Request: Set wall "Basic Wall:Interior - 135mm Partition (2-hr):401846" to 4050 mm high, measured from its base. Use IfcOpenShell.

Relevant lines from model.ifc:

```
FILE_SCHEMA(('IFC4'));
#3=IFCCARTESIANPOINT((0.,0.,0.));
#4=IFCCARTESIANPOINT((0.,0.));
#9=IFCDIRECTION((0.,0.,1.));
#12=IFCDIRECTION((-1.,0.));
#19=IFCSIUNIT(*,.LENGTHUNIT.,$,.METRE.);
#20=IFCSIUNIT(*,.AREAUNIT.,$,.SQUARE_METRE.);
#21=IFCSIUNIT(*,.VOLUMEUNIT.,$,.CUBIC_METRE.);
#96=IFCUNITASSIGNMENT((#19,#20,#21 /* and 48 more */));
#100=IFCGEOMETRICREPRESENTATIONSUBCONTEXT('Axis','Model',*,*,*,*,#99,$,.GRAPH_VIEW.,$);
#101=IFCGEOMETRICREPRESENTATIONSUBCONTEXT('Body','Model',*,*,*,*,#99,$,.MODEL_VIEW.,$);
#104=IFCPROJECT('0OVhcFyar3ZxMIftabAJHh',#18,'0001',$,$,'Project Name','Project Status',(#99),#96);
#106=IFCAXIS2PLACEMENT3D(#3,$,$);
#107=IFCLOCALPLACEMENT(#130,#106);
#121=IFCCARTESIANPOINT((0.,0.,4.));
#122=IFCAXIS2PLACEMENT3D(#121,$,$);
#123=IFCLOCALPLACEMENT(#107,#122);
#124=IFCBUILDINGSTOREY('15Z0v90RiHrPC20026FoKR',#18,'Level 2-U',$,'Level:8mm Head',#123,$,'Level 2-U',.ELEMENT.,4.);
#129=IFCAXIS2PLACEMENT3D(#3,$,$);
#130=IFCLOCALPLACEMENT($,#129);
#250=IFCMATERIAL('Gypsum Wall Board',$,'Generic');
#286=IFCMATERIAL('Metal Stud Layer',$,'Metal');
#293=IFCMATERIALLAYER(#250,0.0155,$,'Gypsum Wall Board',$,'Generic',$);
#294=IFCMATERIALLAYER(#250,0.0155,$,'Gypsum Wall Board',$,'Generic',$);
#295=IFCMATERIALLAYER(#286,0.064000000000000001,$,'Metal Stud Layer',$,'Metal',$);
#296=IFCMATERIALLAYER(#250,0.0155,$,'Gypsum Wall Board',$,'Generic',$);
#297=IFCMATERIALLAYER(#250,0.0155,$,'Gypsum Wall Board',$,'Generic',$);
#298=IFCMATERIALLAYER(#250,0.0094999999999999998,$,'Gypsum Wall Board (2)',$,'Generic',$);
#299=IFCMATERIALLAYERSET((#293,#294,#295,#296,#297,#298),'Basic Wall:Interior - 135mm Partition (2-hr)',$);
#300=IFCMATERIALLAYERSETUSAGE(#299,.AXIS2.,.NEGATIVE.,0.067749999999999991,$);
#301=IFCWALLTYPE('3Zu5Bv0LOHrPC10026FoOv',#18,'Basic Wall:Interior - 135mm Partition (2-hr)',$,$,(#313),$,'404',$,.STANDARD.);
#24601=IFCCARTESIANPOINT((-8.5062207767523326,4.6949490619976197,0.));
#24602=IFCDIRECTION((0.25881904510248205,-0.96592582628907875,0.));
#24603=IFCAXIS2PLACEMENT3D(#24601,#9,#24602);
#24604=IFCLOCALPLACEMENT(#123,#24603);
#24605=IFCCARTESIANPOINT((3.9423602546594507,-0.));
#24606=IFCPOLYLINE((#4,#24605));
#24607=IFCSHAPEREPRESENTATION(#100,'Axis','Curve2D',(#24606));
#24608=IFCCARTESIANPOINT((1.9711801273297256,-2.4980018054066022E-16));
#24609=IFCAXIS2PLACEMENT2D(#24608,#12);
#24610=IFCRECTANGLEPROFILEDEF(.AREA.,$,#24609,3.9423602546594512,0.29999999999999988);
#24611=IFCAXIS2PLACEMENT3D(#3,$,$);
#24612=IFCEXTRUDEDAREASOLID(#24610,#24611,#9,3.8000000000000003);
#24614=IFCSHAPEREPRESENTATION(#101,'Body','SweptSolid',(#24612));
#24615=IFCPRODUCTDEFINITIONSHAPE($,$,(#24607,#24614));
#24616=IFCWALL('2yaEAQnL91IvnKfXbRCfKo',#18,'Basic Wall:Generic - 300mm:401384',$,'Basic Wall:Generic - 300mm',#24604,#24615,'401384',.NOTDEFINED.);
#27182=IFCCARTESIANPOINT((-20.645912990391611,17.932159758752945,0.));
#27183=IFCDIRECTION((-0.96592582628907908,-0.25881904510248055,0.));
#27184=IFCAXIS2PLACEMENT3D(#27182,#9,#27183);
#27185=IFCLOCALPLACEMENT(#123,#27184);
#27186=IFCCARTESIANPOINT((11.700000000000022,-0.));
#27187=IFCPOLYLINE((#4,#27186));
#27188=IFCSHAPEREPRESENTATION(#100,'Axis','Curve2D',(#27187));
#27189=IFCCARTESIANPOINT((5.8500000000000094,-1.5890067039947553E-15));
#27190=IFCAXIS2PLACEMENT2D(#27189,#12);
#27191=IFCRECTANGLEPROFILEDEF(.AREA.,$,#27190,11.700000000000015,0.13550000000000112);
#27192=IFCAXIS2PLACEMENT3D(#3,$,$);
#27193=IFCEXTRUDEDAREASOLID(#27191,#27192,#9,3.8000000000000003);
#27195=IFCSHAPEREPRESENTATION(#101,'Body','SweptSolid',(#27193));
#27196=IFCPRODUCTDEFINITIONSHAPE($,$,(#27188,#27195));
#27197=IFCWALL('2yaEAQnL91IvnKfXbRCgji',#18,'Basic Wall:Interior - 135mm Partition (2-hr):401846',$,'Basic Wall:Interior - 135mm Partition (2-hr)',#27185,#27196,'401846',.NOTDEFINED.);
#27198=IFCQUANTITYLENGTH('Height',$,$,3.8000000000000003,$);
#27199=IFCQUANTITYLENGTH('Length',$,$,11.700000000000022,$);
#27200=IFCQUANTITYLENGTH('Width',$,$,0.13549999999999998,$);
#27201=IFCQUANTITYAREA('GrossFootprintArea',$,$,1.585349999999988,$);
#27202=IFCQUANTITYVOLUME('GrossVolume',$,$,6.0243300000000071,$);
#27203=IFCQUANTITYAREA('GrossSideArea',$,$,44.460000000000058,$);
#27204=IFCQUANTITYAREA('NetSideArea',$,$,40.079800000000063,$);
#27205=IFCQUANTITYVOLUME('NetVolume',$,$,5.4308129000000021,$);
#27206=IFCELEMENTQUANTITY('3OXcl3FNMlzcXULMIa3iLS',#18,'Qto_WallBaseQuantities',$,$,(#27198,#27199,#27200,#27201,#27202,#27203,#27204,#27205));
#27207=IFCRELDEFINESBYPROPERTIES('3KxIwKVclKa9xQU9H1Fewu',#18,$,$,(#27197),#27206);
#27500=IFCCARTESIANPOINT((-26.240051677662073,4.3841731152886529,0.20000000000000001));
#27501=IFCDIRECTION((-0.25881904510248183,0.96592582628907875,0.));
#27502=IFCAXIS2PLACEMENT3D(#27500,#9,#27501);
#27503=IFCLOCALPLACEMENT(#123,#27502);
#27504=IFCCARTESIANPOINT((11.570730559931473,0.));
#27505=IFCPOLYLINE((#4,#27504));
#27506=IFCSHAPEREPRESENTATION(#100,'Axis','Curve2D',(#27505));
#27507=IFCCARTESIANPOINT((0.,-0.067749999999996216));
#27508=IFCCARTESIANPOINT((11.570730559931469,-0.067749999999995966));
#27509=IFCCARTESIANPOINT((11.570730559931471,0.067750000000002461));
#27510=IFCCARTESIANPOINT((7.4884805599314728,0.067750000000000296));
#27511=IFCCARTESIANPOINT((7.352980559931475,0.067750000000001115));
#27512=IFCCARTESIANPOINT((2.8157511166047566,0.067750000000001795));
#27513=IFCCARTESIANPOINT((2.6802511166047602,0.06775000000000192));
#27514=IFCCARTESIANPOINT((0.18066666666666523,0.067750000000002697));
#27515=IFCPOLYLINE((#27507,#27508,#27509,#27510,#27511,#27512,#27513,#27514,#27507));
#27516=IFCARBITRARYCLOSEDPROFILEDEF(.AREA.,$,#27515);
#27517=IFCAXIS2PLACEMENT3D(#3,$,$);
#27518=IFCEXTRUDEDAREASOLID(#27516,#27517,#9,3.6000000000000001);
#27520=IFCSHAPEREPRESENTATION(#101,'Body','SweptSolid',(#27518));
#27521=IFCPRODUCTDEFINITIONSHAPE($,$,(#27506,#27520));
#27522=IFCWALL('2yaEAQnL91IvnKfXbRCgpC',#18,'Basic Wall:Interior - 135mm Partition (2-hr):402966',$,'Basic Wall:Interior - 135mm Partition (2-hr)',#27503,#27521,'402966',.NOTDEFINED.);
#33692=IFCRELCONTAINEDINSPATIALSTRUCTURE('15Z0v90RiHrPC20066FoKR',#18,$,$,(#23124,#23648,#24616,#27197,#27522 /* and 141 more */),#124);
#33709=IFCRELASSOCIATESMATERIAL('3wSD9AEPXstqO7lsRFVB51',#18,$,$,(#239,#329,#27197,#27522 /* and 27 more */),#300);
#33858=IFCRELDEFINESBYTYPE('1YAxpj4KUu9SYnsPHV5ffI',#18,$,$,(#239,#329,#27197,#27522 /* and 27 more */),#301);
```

```python
import ifcopenshell
import ifcopenshell.api.pset
import ifcopenshell.geom
import ifcopenshell.util.element
import ifcopenshell.util.representation
import ifcopenshell.util.shape
import ifcopenshell.util.unit

model = ifcopenshell.open("model.ifc")
unit_scale = ifcopenshell.util.unit.calculate_unit_scale(model)
area_scale = ifcopenshell.util.unit.calculate_unit_scale(model, "AREAUNIT")
volume_scale = ifcopenshell.util.unit.calculate_unit_scale(model, "VOLUMEUNIT")
settings = ifcopenshell.geom.settings()


def volume(element):
    """Net volume in cubic metres, openings subtracted."""
    shape = ifcopenshell.geom.create_shape(settings, element)
    return ifcopenshell.util.shape.get_volume(shape.geometry)


wall = model.by_guid("2yaEAQnL91IvnKfXbRCgji")
before = volume(wall)

body = ifcopenshell.util.representation.get_representation(wall, "Model", "Body")
solid = body.Items[0]
old_height = solid.Depth
solid.Depth = 4.05 / unit_scale
after = volume(wall)
thickness = 0.1355  # wall thickness in metres

# Update the stored height, areas and volumes.
qto = model.by_id(ifcopenshell.util.element.get_pset(wall, "Qto_WallBaseQuantities", should_inherit=False)["id"])
ifcopenshell.api.pset.edit_qto(model, qto=qto, properties={
    "Height": solid.Depth,
    "GrossVolume": ifcopenshell.util.element.get_pset(wall, "Qto_WallBaseQuantities", "GrossVolume") * solid.Depth / old_height,
    "GrossSideArea": ifcopenshell.util.element.get_pset(wall, "Qto_WallBaseQuantities", "GrossSideArea") * solid.Depth / old_height,
    "NetSideArea": after / thickness / area_scale,
    "NetVolume": after / volume_scale,
})

print(f"height {old_height:g} -> {solid.Depth:g}, volume {before:.3f} -> {after:.3f} m3")

model.write("model_updated.ifc")
```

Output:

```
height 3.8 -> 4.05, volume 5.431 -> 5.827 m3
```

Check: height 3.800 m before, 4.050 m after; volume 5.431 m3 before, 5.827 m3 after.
